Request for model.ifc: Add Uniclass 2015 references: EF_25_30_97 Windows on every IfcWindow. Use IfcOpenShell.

First a look at what the model holds.

```python
import ifcopenshell

model = ifcopenshell.open("model.ifc")
print(model.schema)
print("classifications:", [c.Name for c in model.by_type("IfcClassification")])
for ifc_class in ("IfcDoor", "IfcRoof", "IfcStair", "IfcWall", "IfcWindow"):
    print(ifc_class, len(model.by_type(ifc_class)))
```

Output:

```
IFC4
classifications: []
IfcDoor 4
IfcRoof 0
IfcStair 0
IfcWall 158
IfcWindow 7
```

```python
import ifcopenshell
import ifcopenshell.api.classification

model = ifcopenshell.open("model.ifc")

system = ifcopenshell.api.classification.add_classification(model, classification="Uniclass 2015")

codes = {
    "IfcWindow": ("EF_25_30_97", "Windows"),
}
for ifc_class, (code, name) in codes.items():
    products = model.by_type(ifc_class)
    ifcopenshell.api.classification.add_reference(
        model, products=products, classification=system, identification=code, name=name
    )
    print(code, len(products))

model.write("model_updated.ifc")
```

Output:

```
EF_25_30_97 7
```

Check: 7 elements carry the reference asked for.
